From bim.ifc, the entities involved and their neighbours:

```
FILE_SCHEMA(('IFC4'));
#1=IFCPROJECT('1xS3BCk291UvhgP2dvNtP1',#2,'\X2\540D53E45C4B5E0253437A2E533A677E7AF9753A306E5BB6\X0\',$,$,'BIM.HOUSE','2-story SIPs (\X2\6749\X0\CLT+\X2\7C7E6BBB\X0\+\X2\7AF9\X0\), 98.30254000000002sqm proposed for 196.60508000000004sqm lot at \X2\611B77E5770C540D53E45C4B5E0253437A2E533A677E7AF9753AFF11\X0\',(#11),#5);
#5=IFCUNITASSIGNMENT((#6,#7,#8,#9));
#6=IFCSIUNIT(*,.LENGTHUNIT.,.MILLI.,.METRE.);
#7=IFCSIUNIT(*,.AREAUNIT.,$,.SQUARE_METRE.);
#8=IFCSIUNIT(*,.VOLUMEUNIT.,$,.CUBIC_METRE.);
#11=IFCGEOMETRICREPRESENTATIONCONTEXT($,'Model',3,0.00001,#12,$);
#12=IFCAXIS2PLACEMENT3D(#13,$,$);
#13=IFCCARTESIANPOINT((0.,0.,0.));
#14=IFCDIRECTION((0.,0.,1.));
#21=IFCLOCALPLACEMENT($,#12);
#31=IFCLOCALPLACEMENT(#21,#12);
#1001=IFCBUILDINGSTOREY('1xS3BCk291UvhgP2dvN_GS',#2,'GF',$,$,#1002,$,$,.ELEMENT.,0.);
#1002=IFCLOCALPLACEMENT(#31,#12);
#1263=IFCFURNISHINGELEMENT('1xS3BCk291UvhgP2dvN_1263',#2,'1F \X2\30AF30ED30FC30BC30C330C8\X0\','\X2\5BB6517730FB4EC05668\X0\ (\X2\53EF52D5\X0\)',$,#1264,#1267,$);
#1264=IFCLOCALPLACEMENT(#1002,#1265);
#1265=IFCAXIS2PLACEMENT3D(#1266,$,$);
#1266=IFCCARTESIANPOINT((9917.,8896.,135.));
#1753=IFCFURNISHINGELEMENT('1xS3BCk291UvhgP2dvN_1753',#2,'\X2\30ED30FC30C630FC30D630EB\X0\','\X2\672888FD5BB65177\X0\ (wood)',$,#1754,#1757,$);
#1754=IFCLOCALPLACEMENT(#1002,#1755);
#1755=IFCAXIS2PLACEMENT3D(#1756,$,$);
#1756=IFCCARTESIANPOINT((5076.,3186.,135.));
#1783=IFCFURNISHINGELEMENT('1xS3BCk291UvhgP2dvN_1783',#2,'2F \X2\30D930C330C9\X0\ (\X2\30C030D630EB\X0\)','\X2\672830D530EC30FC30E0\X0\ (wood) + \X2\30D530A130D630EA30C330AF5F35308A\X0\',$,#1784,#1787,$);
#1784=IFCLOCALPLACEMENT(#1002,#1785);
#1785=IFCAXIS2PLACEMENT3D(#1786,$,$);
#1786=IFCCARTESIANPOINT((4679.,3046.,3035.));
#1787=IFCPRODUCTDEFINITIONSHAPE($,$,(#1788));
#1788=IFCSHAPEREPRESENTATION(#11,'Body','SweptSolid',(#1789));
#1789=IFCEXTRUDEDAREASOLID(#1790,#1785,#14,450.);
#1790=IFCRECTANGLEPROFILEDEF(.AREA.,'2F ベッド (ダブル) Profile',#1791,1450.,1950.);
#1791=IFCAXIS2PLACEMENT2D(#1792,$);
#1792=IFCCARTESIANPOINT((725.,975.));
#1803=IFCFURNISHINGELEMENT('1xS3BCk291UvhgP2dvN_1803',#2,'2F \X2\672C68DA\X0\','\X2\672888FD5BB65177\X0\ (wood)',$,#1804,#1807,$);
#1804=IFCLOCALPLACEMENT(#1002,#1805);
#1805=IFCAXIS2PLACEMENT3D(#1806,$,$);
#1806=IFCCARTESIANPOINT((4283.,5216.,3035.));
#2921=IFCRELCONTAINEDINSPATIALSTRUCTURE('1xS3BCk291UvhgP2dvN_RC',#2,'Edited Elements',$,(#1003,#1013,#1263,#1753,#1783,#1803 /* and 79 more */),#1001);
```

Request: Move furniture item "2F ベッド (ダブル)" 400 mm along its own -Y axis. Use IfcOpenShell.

```python
import ifcopenshell
import ifcopenshell.api.geometry
import ifcopenshell.util.placement
import ifcopenshell.util.unit

model = ifcopenshell.open("bim.ifc")
unit_scale = ifcopenshell.util.unit.calculate_unit_scale(model)

item = model.by_guid("1xS3BCk291UvhgP2dvN_1783")
matrix = ifcopenshell.util.placement.get_local_placement(item.ObjectPlacement)
matrix[:3, 3] -= matrix[:3, 1] * 0.4 / unit_scale
ifcopenshell.api.geometry.edit_object_placement(model, product=item, matrix=matrix, is_si=False)

print(ifcopenshell.util.placement.get_local_placement(item.ObjectPlacement).round(3) + 0.0)

model.write("bim_rev.ifc")
```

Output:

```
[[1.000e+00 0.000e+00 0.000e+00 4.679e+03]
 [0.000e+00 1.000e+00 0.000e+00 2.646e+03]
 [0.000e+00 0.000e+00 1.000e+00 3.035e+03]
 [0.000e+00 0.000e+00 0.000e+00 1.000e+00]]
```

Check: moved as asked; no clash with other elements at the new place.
